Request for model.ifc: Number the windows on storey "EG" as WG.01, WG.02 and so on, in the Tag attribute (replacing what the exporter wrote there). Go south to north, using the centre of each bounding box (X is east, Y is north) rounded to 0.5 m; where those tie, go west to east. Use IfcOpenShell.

First a look at what the model holds.

```python
import ifcopenshell
import ifcopenshell.util.element
import ifcopenshell.util.placement

model = ifcopenshell.open("model.ifc")
print(model.schema)
storey = next(s for s in model.by_type("IfcBuildingStorey") if s.Name == "EG")
windows = [e for e in ifcopenshell.util.element.get_decomposition(storey) if e.is_a("IfcWindow")]
for e in sorted(windows, key=lambda e: e.id()):
    origin = ifcopenshell.util.placement.get_local_placement(e.ObjectPlacement)[:3, 3]
    print(e.id(), e.Tag, e.Name, origin.round(2) + 0.0, sep=" | ")
```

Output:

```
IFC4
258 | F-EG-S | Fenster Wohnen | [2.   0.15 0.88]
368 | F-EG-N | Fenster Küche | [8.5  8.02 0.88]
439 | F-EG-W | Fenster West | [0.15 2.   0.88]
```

```python
import ifcopenshell
import ifcopenshell.geom
import ifcopenshell.util.element
import ifcopenshell.util.shape

model = ifcopenshell.open("model.ifc")
settings = ifcopenshell.geom.settings()
settings.set("use-world-coords", True)


def centre(element):
    shape = ifcopenshell.geom.create_shape(settings, element)
    return ifcopenshell.util.shape.get_bbox_centroid(shape.geometry)


storey = next(s for s in model.by_type("IfcBuildingStorey") if s.Name == "EG")
windows = [e for e in ifcopenshell.util.element.get_decomposition(storey) if e.is_a("IfcWindow")]

# Insertion points can sit at a corner or the storey origin, so sort by the geometry (in metres).
centres = {e: centre(e) for e in windows}
windows.sort(key=lambda e: (round(centres[e][1] / 0.5), centres[e][0]))

for i, e in enumerate(windows, start=1):
    number = f"WG.{i:02d}"
    e.Tag = number
    print(e.id(), number)

model.write("model-out.ifc")
```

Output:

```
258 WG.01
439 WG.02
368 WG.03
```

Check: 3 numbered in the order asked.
